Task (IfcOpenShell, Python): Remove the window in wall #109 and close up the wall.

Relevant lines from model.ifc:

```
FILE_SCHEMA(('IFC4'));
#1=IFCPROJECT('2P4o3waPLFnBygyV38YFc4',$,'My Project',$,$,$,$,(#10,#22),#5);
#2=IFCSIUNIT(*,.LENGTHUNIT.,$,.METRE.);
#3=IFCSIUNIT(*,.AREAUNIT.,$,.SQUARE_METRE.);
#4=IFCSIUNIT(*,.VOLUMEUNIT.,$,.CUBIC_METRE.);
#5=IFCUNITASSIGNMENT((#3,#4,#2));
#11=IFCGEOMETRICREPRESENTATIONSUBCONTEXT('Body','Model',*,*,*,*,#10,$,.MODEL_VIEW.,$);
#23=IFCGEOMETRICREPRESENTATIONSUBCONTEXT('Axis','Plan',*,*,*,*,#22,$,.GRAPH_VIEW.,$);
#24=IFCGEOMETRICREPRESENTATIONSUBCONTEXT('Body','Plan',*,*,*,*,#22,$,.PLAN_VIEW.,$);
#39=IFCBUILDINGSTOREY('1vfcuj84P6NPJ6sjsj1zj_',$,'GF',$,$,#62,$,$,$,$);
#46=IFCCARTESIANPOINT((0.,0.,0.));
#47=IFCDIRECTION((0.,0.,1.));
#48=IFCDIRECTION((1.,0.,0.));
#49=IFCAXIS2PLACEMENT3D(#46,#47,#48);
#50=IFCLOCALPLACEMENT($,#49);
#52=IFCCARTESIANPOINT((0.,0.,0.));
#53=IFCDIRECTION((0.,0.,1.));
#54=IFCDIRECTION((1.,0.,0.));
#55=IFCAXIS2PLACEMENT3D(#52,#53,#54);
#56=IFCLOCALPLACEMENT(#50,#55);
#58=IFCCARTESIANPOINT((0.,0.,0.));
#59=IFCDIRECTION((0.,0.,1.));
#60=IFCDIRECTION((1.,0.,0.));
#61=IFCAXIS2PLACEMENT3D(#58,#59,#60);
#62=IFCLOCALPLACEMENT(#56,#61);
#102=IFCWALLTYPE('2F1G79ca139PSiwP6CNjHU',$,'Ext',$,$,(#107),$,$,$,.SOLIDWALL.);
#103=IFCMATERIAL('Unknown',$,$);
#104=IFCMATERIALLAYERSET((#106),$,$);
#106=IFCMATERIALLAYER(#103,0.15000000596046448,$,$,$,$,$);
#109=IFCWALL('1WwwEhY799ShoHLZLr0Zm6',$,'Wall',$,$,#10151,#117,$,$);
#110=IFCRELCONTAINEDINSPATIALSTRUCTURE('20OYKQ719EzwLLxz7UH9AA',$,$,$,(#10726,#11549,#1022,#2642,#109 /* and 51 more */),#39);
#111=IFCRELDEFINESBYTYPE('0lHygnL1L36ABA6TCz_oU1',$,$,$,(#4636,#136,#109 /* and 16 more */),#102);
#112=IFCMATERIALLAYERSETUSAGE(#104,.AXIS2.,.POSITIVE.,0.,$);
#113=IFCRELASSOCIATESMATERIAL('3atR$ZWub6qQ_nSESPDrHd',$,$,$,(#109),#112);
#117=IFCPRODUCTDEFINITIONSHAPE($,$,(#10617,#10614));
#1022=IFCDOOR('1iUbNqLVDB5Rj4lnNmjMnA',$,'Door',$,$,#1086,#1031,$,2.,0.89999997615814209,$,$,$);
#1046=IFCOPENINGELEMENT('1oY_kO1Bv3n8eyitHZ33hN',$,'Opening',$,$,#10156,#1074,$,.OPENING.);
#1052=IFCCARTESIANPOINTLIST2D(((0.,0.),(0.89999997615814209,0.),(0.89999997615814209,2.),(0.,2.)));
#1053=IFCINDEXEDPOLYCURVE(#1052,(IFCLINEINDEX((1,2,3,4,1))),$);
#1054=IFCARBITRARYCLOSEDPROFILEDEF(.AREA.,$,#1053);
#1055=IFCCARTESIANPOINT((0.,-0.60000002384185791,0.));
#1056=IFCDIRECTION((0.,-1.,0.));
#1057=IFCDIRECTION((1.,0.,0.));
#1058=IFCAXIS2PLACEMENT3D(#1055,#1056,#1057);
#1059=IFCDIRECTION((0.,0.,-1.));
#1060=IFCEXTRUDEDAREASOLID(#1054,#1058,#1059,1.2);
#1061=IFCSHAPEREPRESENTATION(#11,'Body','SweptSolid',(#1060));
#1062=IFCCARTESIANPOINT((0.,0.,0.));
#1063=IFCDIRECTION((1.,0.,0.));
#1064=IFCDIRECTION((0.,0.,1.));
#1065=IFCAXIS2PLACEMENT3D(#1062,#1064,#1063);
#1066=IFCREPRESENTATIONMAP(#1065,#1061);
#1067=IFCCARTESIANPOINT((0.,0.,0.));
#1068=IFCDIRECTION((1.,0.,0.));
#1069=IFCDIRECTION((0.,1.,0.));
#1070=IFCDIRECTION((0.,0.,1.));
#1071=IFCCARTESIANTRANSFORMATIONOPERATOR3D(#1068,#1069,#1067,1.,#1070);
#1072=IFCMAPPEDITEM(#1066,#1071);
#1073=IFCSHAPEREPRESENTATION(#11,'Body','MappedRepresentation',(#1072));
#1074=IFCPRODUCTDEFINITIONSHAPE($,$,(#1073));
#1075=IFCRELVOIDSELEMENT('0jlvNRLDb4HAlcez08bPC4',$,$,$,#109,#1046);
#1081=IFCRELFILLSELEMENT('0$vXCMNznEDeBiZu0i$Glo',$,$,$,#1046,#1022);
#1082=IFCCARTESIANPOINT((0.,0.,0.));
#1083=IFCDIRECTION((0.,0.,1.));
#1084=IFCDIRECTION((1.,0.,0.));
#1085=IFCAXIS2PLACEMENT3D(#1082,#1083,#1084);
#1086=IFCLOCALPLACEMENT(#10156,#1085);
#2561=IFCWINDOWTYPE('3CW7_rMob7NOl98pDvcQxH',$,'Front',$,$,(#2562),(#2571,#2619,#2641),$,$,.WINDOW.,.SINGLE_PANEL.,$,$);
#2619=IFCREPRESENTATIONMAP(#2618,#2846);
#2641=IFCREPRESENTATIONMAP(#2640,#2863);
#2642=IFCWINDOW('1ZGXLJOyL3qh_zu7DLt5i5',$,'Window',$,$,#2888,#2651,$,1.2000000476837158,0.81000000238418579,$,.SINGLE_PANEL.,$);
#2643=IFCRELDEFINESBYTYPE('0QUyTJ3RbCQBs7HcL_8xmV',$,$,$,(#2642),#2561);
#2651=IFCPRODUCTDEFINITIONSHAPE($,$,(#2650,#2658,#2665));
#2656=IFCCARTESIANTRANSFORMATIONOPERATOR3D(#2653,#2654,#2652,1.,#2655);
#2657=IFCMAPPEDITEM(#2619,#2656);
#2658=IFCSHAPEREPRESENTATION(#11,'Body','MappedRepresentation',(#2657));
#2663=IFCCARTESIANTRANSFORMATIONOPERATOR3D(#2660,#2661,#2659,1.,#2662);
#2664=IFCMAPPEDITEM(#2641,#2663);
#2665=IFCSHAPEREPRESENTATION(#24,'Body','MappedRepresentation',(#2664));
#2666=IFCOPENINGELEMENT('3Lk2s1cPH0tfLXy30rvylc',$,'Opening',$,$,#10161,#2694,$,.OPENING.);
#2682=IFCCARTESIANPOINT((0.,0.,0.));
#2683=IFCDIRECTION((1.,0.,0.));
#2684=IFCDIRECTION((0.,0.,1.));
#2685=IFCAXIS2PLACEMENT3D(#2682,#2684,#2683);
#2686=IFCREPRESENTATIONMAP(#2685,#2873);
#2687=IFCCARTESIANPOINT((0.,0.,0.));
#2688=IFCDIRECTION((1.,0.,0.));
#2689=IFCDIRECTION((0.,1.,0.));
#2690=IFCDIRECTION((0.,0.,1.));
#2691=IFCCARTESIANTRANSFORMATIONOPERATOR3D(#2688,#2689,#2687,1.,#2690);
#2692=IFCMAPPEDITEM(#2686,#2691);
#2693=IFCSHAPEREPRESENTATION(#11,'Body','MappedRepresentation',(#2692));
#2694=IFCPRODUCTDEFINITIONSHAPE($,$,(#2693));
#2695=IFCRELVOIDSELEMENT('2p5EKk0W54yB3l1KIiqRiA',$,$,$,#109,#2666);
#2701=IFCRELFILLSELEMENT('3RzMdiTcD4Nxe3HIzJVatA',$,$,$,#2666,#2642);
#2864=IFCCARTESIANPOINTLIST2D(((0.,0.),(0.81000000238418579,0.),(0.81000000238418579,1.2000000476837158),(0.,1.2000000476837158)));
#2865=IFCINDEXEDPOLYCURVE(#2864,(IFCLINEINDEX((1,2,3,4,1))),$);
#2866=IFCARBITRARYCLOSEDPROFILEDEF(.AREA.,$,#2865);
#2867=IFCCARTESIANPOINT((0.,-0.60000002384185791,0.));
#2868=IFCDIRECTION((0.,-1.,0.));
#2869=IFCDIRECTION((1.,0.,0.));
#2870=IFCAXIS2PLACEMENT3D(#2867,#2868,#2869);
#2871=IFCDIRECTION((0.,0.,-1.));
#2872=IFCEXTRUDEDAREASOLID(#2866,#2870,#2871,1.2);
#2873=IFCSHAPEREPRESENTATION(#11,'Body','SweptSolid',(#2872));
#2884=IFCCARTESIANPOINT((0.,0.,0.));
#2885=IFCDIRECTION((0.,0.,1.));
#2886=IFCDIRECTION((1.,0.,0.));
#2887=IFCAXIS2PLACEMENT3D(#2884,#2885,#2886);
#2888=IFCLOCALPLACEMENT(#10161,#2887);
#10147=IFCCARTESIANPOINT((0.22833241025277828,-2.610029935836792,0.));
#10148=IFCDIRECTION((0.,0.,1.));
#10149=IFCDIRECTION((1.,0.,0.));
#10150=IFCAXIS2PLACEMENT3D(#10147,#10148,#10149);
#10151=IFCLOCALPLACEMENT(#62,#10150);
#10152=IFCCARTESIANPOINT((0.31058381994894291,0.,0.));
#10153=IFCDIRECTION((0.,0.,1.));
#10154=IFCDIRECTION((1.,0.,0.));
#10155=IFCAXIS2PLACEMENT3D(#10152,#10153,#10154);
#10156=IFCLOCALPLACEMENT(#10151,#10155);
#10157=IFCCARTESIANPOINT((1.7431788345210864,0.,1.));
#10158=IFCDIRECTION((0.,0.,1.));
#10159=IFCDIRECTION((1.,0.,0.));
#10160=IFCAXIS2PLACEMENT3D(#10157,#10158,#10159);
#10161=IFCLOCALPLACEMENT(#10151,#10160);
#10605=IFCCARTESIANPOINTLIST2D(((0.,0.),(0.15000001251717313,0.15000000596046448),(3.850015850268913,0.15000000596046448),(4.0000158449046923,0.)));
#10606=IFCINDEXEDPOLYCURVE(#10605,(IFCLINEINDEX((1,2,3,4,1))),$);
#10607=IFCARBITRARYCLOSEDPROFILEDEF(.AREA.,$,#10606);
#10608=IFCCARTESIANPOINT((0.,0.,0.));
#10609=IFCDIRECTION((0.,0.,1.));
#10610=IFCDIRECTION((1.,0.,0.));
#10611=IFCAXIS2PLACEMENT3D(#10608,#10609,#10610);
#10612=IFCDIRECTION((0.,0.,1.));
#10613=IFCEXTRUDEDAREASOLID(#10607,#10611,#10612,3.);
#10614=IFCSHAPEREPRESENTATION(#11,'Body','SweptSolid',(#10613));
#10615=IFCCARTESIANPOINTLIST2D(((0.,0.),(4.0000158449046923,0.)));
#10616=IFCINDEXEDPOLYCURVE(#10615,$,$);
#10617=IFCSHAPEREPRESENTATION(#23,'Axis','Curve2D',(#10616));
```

```python
import ifcopenshell
import ifcopenshell.api.feature
import ifcopenshell.api.root
import ifcopenshell.geom
import ifcopenshell.util.shape

model = ifcopenshell.open("model.ifc")
settings = ifcopenshell.geom.settings()


def volume(element):
    """Net volume in cubic metres, openings subtracted."""
    shape = ifcopenshell.geom.create_shape(settings, element)
    return ifcopenshell.util.shape.get_volume(shape.geometry)


window = model.by_guid("1ZGXLJOyL3qh_zu7DLt5i5")
opening = window.FillsVoids[0].RelatingOpeningElement
wall = opening.VoidsElements[0].RelatingBuildingElement
before = volume(wall)

ifcopenshell.api.root.remove_product(model, product=window)
ifcopenshell.api.feature.remove_feature(model, feature=opening)

after = volume(wall)

print(f"wall volume {before:.3f} -> {after:.3f} m3")

model.write("model_edited.ifc")
```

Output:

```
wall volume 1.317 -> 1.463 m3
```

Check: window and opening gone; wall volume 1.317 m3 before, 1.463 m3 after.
